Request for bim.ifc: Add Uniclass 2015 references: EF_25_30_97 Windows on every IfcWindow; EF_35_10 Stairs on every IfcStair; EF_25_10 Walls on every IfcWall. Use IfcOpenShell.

First a look at what the model holds.

```python
import ifcopenshell

model = ifcopenshell.open("bim.ifc")
print(model.schema)
print("classifications:", [c.Name for c in model.by_type("IfcClassification")])
for ifc_class in ("IfcDoor", "IfcRoof", "IfcStair", "IfcWall", "IfcWindow"):
    print(ifc_class, len(model.by_type(ifc_class)))
```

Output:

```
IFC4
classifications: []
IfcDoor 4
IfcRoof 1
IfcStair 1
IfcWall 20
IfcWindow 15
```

```python
import ifcopenshell
import ifcopenshell.api.classification

model = ifcopenshell.open("bim.ifc")

system = ifcopenshell.api.classification.add_classification(model, classification="Uniclass 2015")

codes = {
    "IfcWindow": ("EF_25_30_97", "Windows"),
    "IfcStair": ("EF_35_10", "Stairs"),
    "IfcWall": ("EF_25_10", "Walls"),
}
for ifc_class, (code, name) in codes.items():
    products = model.by_type(ifc_class)
    ifcopenshell.api.classification.add_reference(
        model, products=products, classification=system, identification=code, name=name
    )
    print(code, len(products))

model.write("bim_v2.ifc")
```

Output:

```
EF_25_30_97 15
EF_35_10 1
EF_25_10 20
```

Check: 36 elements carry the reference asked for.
